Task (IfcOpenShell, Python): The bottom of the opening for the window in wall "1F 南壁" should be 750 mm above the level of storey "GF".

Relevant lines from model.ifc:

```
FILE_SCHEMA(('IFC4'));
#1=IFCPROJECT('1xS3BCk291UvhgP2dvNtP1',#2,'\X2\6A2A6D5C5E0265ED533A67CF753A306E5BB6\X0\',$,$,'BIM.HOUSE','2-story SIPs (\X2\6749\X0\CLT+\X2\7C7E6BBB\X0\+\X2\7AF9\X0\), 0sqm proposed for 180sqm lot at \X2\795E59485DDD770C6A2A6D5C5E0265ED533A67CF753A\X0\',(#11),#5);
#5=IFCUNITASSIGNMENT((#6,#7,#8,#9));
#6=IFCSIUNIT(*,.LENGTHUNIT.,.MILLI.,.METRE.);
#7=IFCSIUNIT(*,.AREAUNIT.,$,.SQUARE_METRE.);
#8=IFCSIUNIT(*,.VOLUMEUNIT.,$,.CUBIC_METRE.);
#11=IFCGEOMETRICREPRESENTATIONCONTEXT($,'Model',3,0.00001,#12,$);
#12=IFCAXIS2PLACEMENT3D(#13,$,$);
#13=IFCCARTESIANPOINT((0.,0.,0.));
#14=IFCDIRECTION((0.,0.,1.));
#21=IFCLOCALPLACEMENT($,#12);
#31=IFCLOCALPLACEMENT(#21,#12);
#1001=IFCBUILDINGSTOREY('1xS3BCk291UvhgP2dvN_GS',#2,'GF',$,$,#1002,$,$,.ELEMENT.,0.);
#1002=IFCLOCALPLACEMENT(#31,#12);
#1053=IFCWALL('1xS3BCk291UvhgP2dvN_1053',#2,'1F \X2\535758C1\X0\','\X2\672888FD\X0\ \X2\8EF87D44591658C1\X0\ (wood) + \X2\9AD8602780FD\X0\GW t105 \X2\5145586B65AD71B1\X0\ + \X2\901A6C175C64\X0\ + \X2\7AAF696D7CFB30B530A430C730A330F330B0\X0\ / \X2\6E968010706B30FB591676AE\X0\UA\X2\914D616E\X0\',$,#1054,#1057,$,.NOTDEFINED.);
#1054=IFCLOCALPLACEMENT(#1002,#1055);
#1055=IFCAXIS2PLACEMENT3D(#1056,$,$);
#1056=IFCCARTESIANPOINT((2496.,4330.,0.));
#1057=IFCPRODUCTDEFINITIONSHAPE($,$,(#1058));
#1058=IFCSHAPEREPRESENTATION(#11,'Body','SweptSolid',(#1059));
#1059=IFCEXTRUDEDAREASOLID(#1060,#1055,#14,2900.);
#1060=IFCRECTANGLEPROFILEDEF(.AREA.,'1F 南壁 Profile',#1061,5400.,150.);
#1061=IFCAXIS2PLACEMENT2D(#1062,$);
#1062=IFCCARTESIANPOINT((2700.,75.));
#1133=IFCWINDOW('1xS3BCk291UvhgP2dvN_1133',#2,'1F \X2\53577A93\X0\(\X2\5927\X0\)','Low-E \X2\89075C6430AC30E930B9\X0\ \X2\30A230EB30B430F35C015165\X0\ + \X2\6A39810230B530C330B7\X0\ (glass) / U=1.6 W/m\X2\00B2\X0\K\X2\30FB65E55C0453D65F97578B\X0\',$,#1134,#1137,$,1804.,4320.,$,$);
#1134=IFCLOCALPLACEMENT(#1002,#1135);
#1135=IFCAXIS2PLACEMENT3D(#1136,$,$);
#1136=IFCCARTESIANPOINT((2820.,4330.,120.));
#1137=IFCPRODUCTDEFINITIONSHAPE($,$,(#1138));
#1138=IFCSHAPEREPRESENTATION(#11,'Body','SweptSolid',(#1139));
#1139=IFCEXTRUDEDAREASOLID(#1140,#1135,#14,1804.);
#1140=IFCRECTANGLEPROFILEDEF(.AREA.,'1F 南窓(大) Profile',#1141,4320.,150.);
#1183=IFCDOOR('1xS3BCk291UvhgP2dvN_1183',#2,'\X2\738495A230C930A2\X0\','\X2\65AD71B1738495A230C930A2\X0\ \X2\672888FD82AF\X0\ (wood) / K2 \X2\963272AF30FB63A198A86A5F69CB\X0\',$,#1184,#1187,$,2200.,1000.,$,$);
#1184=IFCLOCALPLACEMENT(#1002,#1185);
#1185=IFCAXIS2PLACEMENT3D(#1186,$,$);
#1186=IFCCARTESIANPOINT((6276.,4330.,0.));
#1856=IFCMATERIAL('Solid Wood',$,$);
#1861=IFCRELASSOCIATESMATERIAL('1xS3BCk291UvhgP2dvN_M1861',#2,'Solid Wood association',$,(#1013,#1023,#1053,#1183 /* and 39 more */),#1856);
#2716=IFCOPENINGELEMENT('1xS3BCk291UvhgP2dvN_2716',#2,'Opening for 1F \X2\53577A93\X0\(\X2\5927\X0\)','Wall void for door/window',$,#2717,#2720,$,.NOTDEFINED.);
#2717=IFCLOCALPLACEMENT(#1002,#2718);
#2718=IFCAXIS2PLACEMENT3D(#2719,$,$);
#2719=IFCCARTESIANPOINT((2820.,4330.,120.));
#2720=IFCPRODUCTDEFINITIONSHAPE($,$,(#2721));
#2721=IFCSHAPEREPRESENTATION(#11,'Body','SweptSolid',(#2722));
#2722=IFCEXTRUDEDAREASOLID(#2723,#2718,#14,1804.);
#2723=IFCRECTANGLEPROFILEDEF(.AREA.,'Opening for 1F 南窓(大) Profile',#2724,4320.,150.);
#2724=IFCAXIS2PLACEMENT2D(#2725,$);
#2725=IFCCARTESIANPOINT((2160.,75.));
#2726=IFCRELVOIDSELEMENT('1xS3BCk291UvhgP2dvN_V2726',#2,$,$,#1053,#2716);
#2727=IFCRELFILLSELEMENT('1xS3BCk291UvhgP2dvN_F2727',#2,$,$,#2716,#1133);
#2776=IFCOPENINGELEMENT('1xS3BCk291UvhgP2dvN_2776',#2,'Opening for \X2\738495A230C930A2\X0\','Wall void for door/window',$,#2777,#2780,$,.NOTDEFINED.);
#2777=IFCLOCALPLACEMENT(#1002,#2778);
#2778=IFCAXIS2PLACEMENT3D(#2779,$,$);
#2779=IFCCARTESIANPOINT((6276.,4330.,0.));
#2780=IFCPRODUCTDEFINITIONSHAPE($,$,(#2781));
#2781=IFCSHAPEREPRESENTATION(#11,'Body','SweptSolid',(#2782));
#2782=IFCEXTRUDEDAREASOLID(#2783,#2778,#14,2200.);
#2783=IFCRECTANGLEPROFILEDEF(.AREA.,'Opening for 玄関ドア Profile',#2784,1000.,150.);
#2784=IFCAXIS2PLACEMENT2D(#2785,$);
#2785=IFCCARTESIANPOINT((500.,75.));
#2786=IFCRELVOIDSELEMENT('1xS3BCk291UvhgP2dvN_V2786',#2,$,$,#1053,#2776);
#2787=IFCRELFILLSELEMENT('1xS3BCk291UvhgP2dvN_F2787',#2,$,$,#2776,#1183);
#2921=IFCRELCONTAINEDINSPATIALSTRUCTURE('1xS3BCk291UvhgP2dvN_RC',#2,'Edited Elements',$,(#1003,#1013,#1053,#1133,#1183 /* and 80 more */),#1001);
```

```python
import numpy as np
import ifcopenshell
import ifcopenshell.api.geometry
import ifcopenshell.geom
import ifcopenshell.util.element
import ifcopenshell.util.placement
import ifcopenshell.util.shape
import ifcopenshell.util.unit

model = ifcopenshell.open("model.ifc")
unit_scale = ifcopenshell.util.unit.calculate_unit_scale(model)

window = model.by_guid("1xS3BCk291UvhgP2dvN_1133")
opening = window.FillsVoids[0].RelatingOpeningElement
storey = ifcopenshell.util.element.get_container(window, ifc_class="IfcBuildingStorey")
level = ifcopenshell.util.placement.get_local_placement(storey.ObjectPlacement)[2, 3]

# The opening's origin need not be at the sill, so measure its lowest point.
shape = ifcopenshell.geom.create_shape(ifcopenshell.geom.settings(), opening)
bottom = ifcopenshell.util.shape.get_shape_bottom_elevation(shape, shape.geometry) / unit_scale
dz = level + 0.75 / unit_scale - bottom

shift = np.array([0.0, 0.0, dz])
# The window is not placed relative to its opening, so move both.
for product in (opening, window):
    matrix = ifcopenshell.util.placement.get_local_placement(product.ObjectPlacement)
    matrix[:3, 3] += shift
    ifcopenshell.api.geometry.edit_object_placement(model, product=product, matrix=matrix, is_si=False)

print(f"moved by {dz * unit_scale:+.3f} m")

model.write("model_updated.ifc")
```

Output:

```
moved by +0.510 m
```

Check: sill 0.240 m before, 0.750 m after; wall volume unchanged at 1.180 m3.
